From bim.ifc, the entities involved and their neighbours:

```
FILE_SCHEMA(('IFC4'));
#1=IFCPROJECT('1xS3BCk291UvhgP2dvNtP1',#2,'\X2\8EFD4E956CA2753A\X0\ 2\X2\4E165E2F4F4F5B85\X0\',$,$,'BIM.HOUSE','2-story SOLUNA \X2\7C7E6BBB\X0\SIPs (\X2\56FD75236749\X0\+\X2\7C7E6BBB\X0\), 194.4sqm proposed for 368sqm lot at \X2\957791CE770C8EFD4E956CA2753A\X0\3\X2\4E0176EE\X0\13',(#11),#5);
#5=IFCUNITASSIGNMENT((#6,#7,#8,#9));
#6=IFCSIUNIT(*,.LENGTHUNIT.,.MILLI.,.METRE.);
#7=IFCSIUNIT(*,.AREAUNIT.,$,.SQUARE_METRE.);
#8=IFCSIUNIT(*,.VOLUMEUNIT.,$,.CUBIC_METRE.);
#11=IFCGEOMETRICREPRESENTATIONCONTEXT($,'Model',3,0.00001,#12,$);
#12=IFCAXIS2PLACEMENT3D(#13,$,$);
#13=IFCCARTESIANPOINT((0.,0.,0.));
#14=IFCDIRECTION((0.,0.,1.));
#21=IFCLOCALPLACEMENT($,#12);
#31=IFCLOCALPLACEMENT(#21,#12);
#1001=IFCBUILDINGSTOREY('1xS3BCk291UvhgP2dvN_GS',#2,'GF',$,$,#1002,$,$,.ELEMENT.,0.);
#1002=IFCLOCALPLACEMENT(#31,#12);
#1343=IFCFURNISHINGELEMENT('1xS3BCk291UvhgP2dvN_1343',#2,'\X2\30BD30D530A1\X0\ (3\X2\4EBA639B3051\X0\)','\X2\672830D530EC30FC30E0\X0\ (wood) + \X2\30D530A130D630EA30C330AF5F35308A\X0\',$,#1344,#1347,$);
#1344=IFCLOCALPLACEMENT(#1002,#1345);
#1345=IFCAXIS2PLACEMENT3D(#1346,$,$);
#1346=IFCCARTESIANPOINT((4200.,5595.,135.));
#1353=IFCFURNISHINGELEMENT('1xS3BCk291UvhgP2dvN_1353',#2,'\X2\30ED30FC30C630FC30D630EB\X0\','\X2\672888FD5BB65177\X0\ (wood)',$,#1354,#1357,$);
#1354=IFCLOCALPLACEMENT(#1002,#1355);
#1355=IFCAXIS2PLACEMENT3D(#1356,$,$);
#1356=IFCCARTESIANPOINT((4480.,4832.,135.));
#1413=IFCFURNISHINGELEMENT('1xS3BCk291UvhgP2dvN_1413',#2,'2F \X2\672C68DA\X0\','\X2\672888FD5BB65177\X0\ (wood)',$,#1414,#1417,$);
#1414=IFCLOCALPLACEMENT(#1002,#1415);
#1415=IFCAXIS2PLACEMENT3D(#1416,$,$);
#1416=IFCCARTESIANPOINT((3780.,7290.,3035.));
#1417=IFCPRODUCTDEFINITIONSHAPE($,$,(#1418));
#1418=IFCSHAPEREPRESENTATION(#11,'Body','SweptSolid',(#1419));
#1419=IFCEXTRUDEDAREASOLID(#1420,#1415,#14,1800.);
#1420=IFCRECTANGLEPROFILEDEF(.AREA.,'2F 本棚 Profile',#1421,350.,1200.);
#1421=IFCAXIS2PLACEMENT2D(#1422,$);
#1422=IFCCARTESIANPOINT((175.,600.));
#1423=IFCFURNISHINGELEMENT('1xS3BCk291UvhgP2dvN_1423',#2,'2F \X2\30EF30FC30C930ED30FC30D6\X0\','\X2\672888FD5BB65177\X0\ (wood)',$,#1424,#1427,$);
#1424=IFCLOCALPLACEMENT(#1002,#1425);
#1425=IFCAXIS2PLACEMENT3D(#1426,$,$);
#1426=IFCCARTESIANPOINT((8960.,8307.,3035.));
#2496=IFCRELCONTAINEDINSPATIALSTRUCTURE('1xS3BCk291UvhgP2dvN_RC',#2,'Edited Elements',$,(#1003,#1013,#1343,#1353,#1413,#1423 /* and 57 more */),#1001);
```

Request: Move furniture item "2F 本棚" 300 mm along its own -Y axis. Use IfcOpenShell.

```python
import ifcopenshell
import ifcopenshell.api.geometry
import ifcopenshell.util.placement
import ifcopenshell.util.unit

model = ifcopenshell.open("bim.ifc")
unit_scale = ifcopenshell.util.unit.calculate_unit_scale(model)

item = model.by_guid("1xS3BCk291UvhgP2dvN_1413")
matrix = ifcopenshell.util.placement.get_local_placement(item.ObjectPlacement)
matrix[:3, 3] -= matrix[:3, 1] * 0.3 / unit_scale
ifcopenshell.api.geometry.edit_object_placement(model, product=item, matrix=matrix, is_si=False)

print(ifcopenshell.util.placement.get_local_placement(item.ObjectPlacement).round(3) + 0.0)

model.write("bim_v2.ifc")
```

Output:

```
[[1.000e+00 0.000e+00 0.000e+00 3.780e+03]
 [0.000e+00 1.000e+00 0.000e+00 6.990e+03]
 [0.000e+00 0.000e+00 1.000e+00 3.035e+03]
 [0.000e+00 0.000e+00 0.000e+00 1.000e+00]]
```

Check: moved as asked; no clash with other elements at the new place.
